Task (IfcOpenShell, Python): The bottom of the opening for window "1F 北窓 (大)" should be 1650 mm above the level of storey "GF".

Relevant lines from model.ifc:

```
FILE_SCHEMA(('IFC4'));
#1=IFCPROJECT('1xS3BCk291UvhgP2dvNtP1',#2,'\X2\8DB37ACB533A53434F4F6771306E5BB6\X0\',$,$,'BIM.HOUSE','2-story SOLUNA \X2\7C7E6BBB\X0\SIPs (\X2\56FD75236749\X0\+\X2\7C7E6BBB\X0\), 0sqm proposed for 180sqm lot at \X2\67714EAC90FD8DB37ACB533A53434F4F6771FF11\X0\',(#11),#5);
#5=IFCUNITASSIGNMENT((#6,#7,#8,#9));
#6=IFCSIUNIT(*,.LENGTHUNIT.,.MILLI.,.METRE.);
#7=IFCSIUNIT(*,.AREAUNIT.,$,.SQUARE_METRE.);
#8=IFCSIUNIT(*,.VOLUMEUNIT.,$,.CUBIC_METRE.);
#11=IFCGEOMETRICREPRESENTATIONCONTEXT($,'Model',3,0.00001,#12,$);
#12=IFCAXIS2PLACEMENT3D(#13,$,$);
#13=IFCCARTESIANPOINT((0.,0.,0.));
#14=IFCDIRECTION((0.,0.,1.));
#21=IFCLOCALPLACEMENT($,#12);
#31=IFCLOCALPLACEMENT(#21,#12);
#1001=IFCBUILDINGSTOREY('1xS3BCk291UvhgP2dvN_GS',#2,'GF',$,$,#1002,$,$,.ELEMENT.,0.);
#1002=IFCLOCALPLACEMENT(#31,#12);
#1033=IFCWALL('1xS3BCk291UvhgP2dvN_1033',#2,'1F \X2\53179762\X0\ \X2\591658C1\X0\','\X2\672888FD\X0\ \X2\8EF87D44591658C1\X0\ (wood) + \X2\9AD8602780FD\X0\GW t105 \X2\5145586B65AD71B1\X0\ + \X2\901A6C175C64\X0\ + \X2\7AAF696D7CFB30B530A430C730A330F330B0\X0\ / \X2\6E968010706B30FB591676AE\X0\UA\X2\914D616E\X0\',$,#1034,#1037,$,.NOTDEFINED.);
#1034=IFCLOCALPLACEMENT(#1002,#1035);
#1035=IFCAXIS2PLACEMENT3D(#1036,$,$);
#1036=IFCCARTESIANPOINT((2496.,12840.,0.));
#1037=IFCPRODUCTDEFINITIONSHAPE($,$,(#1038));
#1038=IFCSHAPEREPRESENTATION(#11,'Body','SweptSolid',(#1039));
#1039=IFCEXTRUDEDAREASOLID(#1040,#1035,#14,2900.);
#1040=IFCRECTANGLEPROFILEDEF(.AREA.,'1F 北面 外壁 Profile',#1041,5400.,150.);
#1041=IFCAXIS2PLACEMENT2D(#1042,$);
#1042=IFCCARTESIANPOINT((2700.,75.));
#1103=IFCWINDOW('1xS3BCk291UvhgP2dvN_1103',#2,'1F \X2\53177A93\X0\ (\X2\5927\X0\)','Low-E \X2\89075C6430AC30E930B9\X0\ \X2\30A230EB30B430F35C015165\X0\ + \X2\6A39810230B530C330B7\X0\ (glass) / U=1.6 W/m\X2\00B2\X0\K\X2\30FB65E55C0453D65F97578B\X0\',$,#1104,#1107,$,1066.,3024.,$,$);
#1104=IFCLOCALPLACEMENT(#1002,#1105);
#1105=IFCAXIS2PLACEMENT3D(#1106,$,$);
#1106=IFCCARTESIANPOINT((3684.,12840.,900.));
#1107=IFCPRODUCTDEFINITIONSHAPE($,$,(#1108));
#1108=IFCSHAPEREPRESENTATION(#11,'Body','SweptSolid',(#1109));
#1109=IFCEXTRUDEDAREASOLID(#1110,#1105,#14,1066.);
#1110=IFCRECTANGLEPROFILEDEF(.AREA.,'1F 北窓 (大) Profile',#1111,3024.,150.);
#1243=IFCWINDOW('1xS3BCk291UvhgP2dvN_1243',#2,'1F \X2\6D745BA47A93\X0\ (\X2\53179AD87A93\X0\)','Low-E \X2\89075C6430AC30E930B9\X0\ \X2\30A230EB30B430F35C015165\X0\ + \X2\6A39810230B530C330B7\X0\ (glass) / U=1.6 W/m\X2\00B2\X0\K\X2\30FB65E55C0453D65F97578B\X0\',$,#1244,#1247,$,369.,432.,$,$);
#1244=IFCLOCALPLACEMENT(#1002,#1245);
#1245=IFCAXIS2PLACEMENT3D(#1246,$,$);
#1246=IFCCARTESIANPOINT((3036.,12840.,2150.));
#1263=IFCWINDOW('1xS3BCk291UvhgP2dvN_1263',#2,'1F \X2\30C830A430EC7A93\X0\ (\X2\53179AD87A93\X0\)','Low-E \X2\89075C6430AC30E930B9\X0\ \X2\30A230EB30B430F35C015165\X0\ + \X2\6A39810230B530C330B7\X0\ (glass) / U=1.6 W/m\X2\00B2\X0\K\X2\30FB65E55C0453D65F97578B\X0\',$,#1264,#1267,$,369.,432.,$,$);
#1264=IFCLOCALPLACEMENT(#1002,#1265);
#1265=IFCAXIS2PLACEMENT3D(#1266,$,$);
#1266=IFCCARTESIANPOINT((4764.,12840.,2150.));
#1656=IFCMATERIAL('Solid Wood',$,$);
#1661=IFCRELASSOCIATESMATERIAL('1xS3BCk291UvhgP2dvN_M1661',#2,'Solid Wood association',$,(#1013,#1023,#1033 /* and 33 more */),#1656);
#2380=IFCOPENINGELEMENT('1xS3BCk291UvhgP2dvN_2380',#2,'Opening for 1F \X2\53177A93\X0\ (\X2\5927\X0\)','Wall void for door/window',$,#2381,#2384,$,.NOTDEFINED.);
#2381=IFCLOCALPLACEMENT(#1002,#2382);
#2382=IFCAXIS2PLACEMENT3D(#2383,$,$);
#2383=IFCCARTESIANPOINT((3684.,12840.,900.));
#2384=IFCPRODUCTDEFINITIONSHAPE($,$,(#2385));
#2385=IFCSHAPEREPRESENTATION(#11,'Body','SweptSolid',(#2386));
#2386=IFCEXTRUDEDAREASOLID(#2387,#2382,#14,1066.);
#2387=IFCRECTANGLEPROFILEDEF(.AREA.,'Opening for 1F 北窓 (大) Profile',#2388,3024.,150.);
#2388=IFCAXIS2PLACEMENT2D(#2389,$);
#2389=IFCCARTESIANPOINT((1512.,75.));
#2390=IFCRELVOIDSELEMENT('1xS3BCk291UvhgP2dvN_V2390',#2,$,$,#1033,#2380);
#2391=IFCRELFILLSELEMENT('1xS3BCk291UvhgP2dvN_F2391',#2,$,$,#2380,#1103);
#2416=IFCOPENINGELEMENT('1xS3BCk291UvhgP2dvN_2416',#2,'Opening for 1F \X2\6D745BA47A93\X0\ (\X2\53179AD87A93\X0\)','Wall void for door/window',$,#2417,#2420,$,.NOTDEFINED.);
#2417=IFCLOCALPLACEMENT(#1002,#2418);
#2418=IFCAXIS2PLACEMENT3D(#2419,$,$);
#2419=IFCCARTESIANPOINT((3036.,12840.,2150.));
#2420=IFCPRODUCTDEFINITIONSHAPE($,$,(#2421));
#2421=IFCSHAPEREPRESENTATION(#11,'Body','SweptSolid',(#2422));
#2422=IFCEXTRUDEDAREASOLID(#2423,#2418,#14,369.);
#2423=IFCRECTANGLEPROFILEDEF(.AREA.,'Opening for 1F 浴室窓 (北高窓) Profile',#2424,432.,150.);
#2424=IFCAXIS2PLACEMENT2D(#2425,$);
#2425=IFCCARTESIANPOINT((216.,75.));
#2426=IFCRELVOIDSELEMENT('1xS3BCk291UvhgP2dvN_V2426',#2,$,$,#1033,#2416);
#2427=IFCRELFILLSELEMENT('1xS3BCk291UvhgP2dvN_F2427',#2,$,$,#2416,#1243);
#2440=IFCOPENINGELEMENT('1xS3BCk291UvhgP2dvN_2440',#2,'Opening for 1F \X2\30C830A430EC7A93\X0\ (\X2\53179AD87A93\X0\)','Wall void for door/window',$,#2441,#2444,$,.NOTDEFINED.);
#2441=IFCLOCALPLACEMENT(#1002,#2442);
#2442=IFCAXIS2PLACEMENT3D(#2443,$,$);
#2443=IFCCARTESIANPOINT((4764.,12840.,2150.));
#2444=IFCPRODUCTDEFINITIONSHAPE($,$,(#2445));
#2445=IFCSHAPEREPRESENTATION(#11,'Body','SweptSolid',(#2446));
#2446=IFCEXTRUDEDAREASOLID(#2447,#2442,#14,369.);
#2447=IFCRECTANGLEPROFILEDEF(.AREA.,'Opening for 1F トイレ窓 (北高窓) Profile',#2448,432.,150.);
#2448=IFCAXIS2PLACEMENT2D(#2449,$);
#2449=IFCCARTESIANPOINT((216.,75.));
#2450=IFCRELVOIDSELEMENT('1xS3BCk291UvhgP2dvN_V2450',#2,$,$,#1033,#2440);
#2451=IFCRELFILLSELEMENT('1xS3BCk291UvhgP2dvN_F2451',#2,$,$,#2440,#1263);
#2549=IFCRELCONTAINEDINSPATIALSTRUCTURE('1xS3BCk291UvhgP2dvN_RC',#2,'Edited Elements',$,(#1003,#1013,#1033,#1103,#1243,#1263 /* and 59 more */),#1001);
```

```python
import numpy as np
import ifcopenshell
import ifcopenshell.api.geometry
import ifcopenshell.geom
import ifcopenshell.util.element
import ifcopenshell.util.placement
import ifcopenshell.util.shape
import ifcopenshell.util.unit

model = ifcopenshell.open("model.ifc")
unit_scale = ifcopenshell.util.unit.calculate_unit_scale(model)

window = model.by_guid("1xS3BCk291UvhgP2dvN_1103")
opening = window.FillsVoids[0].RelatingOpeningElement
storey = ifcopenshell.util.element.get_container(window, ifc_class="IfcBuildingStorey")
level = ifcopenshell.util.placement.get_local_placement(storey.ObjectPlacement)[2, 3]

# The opening's origin need not be at the sill, so measure its lowest point.
shape = ifcopenshell.geom.create_shape(ifcopenshell.geom.settings(), opening)
bottom = ifcopenshell.util.shape.get_shape_bottom_elevation(shape, shape.geometry) / unit_scale
dz = level + 1650.0 - bottom

shift = np.array([0.0, 0.0, dz])
# The window is not placed relative to its opening, so move both.
for product in (opening, window):
    matrix = ifcopenshell.util.placement.get_local_placement(product.ObjectPlacement)
    matrix[:3, 3] += shift
    ifcopenshell.api.geometry.edit_object_placement(model, product=product, matrix=matrix, is_si=False)

print(f"moved by {dz * unit_scale:+.3f} m")

model.write("model_v2.ifc")
```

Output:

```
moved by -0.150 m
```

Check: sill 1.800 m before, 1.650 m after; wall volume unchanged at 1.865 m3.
